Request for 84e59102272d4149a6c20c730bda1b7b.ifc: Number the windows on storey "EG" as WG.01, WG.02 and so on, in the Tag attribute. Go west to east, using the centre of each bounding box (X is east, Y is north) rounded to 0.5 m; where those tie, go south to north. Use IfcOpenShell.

First a look at what the model holds.

```python
import ifcopenshell
import ifcopenshell.util.element
import ifcopenshell.util.placement

model = ifcopenshell.open("84e59102272d4149a6c20c730bda1b7b.ifc")
print(model.schema)
storey = next(s for s in model.by_type("IfcBuildingStorey") if s.Name == "EG")
windows = [e for e in ifcopenshell.util.element.get_decomposition(storey) if e.is_a("IfcWindow")]
for e in sorted(windows, key=lambda e: e.id()):
    origin = ifcopenshell.util.placement.get_local_placement(e.ObjectPlacement)[:3, 3]
    print(e.id(), e.Tag, e.Name, origin.round(2) + 0.0, sep=" | ")
```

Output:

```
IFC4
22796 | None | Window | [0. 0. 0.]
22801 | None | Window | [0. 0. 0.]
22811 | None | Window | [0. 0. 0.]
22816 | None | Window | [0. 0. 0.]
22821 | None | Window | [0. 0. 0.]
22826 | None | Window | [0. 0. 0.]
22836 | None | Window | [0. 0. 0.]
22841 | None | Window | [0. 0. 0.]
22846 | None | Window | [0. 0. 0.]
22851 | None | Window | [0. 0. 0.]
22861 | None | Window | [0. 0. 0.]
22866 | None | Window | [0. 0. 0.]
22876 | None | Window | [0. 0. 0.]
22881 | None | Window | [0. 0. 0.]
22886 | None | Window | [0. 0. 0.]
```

```python
import ifcopenshell
import ifcopenshell.geom
import ifcopenshell.util.element
import ifcopenshell.util.shape

model = ifcopenshell.open("84e59102272d4149a6c20c730bda1b7b.ifc")
settings = ifcopenshell.geom.settings()
settings.set("use-world-coords", True)


def centre(element):
    shape = ifcopenshell.geom.create_shape(settings, element)
    return ifcopenshell.util.shape.get_bbox_centroid(shape.geometry)


storey = next(s for s in model.by_type("IfcBuildingStorey") if s.Name == "EG")
windows = [e for e in ifcopenshell.util.element.get_decomposition(storey) if e.is_a("IfcWindow")]

# Insertion points can sit at a corner or the storey origin, so sort by the geometry (in metres).
centres = {e: centre(e) for e in windows}
windows.sort(key=lambda e: (round(centres[e][0] / 0.5), centres[e][1]))

for i, e in enumerate(windows, start=1):
    number = f"WG.{i:02d}"
    e.Tag = number
    print(e.id(), number)

model.write("84e59102272d4149a6c20c730bda1b7b_v2.ifc")
```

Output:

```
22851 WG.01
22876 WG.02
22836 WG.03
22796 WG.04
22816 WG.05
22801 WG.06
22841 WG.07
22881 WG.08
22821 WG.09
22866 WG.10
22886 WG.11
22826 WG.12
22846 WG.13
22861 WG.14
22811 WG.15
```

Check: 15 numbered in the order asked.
